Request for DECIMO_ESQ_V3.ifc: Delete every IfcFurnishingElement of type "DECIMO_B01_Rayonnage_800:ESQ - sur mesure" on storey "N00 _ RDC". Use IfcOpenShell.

First a look at what the model holds.

```python
import ifcopenshell
import ifcopenshell.util.element

model = ifcopenshell.open("DECIMO_ESQ_V3.ifc")
print(model.schema)
storey = next(s for s in model.by_type("IfcBuildingStorey") if s.Name == "N00 _ RDC")
furniture = [e for e in ifcopenshell.util.element.get_decomposition(storey) if e.is_a("IfcFurnishingElement")]
seen = {}
for e in furniture:
    element_type = ifcopenshell.util.element.get_type(e)
    name = element_type.Name if element_type not in (None, e) else None
    seen[name] = seen.get(name, 0) + 1
for name, count in sorted(seen.items(), key=str):
    print(count, "x", name)
```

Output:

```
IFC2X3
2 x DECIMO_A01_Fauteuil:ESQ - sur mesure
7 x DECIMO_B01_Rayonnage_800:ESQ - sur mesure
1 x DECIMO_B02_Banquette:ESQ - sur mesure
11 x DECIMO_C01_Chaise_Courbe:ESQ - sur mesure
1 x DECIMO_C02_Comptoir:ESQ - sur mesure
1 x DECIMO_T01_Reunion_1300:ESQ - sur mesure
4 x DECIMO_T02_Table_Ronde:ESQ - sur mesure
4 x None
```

```python
import ifcopenshell
import ifcopenshell.api.root
import ifcopenshell.util.element

model = ifcopenshell.open("DECIMO_ESQ_V3.ifc")

storey = next(s for s in model.by_type("IfcBuildingStorey") if s.Name == "N00 _ RDC")
furniture = [e for e in ifcopenshell.util.element.get_decomposition(storey) if e.is_a("IfcFurnishingElement")]
targets = [e for e in furniture if (t := ifcopenshell.util.element.get_type(e)) not in (None, e) and t.Name == "DECIMO_B01_Rayonnage_800:ESQ - sur mesure"]

for e in targets:
    ifcopenshell.api.root.remove_product(model, product=e)
print(len(targets), "removed")

model.write("DECIMO_ESQ_V3-out.ifc")
```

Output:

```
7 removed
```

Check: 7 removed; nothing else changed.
